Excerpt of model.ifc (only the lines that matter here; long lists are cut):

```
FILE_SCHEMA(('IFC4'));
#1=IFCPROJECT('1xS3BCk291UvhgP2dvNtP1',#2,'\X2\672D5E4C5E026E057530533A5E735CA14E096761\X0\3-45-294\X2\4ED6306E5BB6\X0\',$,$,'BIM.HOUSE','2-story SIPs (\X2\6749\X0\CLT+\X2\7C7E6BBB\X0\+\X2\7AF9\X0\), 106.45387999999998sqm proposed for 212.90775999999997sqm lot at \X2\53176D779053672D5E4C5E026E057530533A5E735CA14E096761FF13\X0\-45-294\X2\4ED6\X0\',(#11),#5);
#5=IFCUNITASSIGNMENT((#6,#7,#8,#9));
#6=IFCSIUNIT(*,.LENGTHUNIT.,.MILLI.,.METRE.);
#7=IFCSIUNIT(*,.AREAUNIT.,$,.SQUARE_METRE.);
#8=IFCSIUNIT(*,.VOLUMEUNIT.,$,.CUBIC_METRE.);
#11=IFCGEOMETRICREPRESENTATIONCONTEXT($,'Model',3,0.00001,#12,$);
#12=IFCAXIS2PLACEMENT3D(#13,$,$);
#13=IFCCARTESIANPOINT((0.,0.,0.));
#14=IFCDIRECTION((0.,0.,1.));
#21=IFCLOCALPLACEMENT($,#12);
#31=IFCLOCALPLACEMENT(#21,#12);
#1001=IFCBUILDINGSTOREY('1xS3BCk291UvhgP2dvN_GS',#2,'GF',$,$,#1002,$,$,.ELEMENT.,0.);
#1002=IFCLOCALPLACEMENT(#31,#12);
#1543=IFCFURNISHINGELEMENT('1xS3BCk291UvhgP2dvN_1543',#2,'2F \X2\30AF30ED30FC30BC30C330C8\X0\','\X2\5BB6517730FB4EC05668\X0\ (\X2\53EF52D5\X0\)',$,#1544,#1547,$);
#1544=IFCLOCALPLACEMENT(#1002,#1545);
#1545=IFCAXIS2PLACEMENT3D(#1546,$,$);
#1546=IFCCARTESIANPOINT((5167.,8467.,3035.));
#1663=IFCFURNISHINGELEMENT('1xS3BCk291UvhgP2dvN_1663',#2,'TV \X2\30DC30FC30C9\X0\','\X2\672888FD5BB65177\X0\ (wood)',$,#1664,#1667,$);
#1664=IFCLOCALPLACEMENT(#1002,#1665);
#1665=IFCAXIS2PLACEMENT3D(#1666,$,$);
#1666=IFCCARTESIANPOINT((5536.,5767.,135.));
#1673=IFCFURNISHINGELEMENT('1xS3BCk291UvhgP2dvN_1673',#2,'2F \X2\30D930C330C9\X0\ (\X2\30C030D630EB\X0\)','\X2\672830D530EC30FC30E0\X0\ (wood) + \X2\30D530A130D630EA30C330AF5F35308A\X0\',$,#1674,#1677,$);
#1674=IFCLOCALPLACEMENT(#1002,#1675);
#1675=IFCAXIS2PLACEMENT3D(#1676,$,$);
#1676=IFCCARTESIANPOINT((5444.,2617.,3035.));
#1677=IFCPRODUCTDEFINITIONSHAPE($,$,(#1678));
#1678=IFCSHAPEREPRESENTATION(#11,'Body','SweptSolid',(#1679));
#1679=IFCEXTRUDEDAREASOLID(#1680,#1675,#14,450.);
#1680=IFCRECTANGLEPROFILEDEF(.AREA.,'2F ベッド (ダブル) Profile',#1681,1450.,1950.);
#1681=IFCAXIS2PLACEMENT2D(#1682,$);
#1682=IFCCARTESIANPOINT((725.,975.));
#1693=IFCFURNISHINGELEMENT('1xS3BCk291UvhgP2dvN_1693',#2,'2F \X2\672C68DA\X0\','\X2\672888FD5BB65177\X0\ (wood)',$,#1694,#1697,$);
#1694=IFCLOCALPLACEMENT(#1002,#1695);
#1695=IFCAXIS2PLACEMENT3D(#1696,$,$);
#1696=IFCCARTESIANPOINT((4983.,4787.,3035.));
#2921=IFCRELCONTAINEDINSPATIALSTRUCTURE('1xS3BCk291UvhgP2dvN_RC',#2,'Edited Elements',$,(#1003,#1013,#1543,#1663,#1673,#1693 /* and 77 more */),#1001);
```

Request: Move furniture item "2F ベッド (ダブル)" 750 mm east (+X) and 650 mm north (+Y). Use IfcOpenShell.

```python
import ifcopenshell
import ifcopenshell.api.geometry
import ifcopenshell.util.placement

model = ifcopenshell.open("model.ifc")

item = model.by_guid("1xS3BCk291UvhgP2dvN_1673")
matrix = ifcopenshell.util.placement.get_local_placement(item.ObjectPlacement)
matrix[0, 3] += 750.0
matrix[1, 3] += 650.0
ifcopenshell.api.geometry.edit_object_placement(model, product=item, matrix=matrix, is_si=False)

print(ifcopenshell.util.placement.get_local_placement(item.ObjectPlacement).round(3) + 0.0)

model.write("model-out.ifc")
```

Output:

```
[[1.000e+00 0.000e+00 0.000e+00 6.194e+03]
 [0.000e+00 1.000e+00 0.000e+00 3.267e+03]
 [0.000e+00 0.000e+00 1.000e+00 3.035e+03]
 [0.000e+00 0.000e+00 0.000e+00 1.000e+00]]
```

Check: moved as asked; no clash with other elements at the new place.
